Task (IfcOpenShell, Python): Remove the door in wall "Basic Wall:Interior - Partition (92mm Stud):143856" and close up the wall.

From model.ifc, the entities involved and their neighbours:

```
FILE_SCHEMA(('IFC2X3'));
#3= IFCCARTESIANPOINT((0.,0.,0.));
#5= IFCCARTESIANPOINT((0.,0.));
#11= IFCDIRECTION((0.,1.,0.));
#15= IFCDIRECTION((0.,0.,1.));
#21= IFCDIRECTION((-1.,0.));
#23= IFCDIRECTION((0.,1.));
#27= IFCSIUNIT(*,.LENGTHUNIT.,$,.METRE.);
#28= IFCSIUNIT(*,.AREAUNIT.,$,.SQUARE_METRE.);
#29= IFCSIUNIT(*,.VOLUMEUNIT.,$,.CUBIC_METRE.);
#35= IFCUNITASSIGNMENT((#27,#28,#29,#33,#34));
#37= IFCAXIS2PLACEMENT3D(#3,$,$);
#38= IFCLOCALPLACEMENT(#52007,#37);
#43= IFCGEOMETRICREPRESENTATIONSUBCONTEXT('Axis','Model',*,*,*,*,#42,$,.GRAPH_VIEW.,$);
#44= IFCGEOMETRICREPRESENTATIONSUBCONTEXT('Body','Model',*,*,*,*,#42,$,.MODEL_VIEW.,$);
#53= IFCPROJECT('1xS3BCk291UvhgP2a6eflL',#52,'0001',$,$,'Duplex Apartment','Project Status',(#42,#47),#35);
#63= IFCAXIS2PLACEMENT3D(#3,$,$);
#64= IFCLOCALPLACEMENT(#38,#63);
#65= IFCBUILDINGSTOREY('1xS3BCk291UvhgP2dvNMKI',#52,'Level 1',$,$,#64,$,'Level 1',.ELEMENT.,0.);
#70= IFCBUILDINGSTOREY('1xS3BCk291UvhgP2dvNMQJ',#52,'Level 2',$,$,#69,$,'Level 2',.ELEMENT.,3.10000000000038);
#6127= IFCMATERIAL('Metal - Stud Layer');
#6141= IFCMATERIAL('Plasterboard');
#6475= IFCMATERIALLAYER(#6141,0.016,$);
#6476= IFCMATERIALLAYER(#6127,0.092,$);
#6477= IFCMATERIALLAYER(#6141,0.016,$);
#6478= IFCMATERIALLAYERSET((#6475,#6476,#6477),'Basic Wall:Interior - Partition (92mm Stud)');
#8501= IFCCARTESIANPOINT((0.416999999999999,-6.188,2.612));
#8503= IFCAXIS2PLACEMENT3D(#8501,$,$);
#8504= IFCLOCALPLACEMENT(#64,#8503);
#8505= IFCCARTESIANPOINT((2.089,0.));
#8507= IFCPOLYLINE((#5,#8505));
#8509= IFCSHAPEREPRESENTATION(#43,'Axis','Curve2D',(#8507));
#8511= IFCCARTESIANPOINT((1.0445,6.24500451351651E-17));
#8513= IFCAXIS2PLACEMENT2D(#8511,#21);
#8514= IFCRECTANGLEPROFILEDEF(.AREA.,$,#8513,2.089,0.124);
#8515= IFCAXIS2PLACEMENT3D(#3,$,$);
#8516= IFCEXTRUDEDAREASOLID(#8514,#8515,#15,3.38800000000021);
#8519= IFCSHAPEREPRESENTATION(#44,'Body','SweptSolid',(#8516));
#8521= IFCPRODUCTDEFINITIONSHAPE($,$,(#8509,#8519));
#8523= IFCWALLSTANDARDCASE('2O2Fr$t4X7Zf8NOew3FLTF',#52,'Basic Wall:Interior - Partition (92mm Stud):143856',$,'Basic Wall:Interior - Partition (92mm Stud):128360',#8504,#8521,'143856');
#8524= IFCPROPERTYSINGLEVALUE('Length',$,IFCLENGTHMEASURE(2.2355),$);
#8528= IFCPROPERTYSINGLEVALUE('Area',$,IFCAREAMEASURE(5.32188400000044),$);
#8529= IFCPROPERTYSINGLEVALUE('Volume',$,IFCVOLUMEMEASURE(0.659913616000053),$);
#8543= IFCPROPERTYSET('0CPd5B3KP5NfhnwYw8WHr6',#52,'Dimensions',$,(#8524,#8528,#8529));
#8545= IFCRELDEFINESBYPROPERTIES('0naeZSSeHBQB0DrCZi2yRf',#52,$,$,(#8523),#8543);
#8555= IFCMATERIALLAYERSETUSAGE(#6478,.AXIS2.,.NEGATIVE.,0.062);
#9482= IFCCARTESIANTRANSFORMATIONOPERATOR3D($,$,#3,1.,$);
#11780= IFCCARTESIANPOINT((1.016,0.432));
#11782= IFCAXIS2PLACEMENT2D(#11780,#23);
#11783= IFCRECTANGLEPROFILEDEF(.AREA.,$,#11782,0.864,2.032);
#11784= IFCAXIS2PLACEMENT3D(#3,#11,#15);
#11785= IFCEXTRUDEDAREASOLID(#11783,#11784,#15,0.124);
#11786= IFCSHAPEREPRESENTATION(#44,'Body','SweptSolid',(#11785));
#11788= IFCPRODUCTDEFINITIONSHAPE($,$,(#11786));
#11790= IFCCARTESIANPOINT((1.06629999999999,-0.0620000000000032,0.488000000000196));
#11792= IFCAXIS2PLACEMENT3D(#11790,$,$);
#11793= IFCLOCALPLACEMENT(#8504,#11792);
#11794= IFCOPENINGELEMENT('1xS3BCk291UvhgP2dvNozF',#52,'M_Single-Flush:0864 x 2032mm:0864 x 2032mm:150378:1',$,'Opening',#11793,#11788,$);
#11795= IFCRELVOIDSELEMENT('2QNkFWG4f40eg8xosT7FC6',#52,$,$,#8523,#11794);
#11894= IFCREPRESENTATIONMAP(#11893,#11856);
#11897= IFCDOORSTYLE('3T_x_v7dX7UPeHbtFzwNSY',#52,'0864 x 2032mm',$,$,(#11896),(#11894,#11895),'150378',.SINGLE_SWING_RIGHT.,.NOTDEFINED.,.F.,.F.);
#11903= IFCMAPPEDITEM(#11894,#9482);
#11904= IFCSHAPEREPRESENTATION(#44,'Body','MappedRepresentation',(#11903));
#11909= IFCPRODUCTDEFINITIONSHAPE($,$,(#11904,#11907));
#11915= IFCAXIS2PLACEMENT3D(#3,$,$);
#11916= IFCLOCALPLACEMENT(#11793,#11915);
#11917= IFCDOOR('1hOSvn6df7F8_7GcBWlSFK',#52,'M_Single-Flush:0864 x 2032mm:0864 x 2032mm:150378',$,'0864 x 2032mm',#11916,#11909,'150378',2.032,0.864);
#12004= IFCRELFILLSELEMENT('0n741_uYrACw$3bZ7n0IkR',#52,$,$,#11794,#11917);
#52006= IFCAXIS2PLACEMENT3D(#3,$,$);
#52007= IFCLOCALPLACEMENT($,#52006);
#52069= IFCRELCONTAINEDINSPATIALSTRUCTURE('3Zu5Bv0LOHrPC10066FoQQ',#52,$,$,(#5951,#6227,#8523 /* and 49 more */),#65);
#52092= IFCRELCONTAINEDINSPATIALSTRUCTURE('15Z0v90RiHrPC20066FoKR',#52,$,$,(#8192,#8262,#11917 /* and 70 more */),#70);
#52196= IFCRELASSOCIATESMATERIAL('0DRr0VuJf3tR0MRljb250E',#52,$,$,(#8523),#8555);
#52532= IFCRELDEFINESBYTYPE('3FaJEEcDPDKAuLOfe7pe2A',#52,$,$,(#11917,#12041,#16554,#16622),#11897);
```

```python
import ifcopenshell
import ifcopenshell.api.feature
import ifcopenshell.api.pset
import ifcopenshell.api.root
import ifcopenshell.geom
import ifcopenshell.util.element
import ifcopenshell.util.shape
import ifcopenshell.util.unit

model = ifcopenshell.open("model.ifc")
area_scale = ifcopenshell.util.unit.calculate_unit_scale(model, "AREAUNIT")
volume_scale = ifcopenshell.util.unit.calculate_unit_scale(model, "VOLUMEUNIT")
settings = ifcopenshell.geom.settings()


def volume(element):
    """Net volume in cubic metres, openings subtracted."""
    shape = ifcopenshell.geom.create_shape(settings, element)
    return ifcopenshell.util.shape.get_volume(shape.geometry)


door = model.by_guid("1hOSvn6df7F8_7GcBWlSFK")
opening = door.FillsVoids[0].RelatingOpeningElement
wall = opening.VoidsElements[0].RelatingBuildingElement
before = volume(wall)

ifcopenshell.api.root.remove_product(model, product=door)
ifcopenshell.api.feature.remove_feature(model, feature=opening)

after = volume(wall)
thickness = 0.124  # wall thickness in metres

# Update the wall's stored quantities.
pset = model.by_id(ifcopenshell.util.element.get_pset(wall, "Dimensions", should_inherit=False)["id"])
ifcopenshell.api.pset.edit_pset(model, pset=pset, properties={
    "Area": model.create_entity("IfcAreaMeasure", after / thickness / area_scale),
    "Volume": model.create_entity("IfcVolumeMeasure", after / volume_scale),
})

print(f"wall volume {before:.3f} -> {after:.3f} m3")

model.write("model_rev.ifc")
```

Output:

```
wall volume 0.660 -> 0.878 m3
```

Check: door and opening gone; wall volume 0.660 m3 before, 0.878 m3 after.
